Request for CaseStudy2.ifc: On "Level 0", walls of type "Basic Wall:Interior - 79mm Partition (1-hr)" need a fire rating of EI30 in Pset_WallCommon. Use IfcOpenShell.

First a look at what the model holds.

```python
import ifcopenshell
import ifcopenshell.util.element

model = ifcopenshell.open("CaseStudy2.ifc")
print(model.schema)
storey = next(s for s in model.by_type("IfcBuildingStorey") if s.Name == "Level 0")
walls = [e for e in ifcopenshell.util.element.get_decomposition(storey) if e.is_a("IfcWall")]
seen = {}
for e in walls:
    element_type = ifcopenshell.util.element.get_type(e)
    key = (element_type.Name if element_type != e and element_type else None, ifcopenshell.util.element.get_pset(e, "Pset_WallCommon", "FireRating"))
    seen[key] = seen.get(key, 0) + 1
for (name, value), count in sorted(seen.items(), key=str):
    print(count, "x", name, "|", value)
```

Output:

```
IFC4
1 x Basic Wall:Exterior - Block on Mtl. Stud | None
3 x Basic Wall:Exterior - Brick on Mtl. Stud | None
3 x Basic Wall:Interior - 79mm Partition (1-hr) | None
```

```python
import ifcopenshell
import ifcopenshell.api.pset
import ifcopenshell.util.element

model = ifcopenshell.open("CaseStudy2.ifc")

storey = next(s for s in model.by_type("IfcBuildingStorey") if s.Name == "Level 0")
walls = [e for e in ifcopenshell.util.element.get_decomposition(storey) if e.is_a("IfcWall")]

count = 0
for e in walls:
    element_type = ifcopenshell.util.element.get_type(e)
    if element_type in (None, e) or element_type.Name != "Basic Wall:Interior - 79mm Partition (1-hr)":
        continue
    # add_pset returns the element's existing set when there is one.
    pset = ifcopenshell.api.pset.add_pset(model, product=e, name="Pset_WallCommon")
    ifcopenshell.api.pset.edit_pset(model, pset=pset, properties={"FireRating": "EI30"})
    count += 1

print(count, "walls updated")

model.write("CaseStudy2_v2.ifc")
```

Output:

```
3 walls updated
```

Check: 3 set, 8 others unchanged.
